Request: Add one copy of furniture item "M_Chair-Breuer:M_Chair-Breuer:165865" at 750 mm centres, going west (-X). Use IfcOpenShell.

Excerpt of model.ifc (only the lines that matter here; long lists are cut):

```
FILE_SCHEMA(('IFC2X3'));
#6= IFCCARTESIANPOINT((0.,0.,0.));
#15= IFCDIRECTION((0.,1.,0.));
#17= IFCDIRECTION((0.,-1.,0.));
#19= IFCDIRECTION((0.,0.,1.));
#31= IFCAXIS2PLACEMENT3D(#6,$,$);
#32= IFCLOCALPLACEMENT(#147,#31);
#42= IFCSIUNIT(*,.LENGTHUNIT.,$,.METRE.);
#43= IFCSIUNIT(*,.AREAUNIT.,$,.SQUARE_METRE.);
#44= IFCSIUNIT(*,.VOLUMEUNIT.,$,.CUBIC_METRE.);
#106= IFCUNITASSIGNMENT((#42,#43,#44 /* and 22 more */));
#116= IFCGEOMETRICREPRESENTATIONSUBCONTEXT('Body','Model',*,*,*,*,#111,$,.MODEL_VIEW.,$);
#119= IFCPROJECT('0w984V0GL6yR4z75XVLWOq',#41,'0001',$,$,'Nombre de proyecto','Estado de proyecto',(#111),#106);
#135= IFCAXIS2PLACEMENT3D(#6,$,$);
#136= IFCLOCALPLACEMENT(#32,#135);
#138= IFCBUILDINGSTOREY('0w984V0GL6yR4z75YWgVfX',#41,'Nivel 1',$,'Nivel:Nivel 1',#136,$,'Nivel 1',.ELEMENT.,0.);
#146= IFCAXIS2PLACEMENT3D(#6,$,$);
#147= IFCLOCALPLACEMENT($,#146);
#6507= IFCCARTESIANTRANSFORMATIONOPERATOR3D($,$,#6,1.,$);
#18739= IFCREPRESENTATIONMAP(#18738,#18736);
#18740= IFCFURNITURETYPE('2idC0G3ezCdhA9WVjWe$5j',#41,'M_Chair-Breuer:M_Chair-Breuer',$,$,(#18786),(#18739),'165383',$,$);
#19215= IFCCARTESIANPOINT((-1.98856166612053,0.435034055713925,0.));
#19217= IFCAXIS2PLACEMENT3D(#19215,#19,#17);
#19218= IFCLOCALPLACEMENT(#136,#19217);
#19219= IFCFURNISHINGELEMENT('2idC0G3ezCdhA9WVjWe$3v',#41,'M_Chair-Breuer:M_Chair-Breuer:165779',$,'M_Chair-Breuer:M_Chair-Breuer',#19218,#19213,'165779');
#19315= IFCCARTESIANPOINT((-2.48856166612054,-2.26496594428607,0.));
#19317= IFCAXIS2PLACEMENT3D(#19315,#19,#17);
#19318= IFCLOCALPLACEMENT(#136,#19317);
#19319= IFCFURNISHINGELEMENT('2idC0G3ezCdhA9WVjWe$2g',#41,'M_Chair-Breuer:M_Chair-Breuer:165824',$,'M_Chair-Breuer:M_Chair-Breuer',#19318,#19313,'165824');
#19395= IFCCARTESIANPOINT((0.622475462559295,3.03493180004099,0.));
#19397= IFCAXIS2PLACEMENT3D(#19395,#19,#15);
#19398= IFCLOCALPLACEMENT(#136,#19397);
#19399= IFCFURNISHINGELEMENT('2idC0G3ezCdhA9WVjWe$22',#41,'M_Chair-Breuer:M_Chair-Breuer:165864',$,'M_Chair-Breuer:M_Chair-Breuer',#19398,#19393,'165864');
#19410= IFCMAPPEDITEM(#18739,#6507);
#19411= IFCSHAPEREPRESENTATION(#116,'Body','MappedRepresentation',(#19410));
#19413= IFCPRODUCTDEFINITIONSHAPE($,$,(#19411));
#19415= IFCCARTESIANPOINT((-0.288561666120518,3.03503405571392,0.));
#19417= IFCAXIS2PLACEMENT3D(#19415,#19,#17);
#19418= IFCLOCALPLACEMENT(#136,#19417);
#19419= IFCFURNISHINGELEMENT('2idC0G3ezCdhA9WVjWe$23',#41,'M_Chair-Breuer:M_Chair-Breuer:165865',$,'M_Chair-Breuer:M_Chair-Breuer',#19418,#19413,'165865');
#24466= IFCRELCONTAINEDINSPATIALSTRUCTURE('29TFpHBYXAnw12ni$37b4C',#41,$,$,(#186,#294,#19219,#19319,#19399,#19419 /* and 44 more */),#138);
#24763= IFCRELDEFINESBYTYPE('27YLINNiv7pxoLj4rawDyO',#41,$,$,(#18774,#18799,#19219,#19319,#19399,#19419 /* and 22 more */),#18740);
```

```python
import numpy as np
import ifcopenshell
import ifcopenshell.api.geometry
import ifcopenshell.api.root
import ifcopenshell.util.element
import ifcopenshell.util.placement
import ifcopenshell.util.unit

model = ifcopenshell.open("model.ifc")
unit_scale = ifcopenshell.util.unit.calculate_unit_scale(model)


def reuse_history(source, copy):
    """copy_class also copies each property set's owner history, people and application; keep the originals."""
    for rel in copy.IsDefinedBy:
        if rel.is_a("IfcRelDefinesByProperties") and (history := rel.RelatingPropertyDefinition.OwnerHistory):
            rel.RelatingPropertyDefinition.OwnerHistory = source.OwnerHistory
            ifcopenshell.util.element.remove_deep2(model, history)


source = model.by_guid("2idC0G3ezCdhA9WVjWe$23")
base = ifcopenshell.util.placement.get_local_placement(source.ObjectPlacement)
step = np.array([-1.0, 0.0, 0.0]) * 0.75 / unit_scale

for i in range(1, 2):
    copy = ifcopenshell.api.root.copy_class(model, product=source)
    copy.Representation = ifcopenshell.util.element.copy_deep(
        model, source.Representation, exclude=["IfcGeometricRepresentationContext", "IfcRepresentationMap"]
    )
    copy.Name = "M_Chair-Breuer:M_Chair-Breuer"
    copy.Tag = None
    reuse_history(source, copy)
    matrix = base.copy()
    matrix[:3, 3] += i * step
    print("added at", matrix[:3, 3].round(3) + 0.0)
    ifcopenshell.api.geometry.edit_object_placement(model, product=copy, matrix=matrix, is_si=False)

model.write("model_v2.ifc")
```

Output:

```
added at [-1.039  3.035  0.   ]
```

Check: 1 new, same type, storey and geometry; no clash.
